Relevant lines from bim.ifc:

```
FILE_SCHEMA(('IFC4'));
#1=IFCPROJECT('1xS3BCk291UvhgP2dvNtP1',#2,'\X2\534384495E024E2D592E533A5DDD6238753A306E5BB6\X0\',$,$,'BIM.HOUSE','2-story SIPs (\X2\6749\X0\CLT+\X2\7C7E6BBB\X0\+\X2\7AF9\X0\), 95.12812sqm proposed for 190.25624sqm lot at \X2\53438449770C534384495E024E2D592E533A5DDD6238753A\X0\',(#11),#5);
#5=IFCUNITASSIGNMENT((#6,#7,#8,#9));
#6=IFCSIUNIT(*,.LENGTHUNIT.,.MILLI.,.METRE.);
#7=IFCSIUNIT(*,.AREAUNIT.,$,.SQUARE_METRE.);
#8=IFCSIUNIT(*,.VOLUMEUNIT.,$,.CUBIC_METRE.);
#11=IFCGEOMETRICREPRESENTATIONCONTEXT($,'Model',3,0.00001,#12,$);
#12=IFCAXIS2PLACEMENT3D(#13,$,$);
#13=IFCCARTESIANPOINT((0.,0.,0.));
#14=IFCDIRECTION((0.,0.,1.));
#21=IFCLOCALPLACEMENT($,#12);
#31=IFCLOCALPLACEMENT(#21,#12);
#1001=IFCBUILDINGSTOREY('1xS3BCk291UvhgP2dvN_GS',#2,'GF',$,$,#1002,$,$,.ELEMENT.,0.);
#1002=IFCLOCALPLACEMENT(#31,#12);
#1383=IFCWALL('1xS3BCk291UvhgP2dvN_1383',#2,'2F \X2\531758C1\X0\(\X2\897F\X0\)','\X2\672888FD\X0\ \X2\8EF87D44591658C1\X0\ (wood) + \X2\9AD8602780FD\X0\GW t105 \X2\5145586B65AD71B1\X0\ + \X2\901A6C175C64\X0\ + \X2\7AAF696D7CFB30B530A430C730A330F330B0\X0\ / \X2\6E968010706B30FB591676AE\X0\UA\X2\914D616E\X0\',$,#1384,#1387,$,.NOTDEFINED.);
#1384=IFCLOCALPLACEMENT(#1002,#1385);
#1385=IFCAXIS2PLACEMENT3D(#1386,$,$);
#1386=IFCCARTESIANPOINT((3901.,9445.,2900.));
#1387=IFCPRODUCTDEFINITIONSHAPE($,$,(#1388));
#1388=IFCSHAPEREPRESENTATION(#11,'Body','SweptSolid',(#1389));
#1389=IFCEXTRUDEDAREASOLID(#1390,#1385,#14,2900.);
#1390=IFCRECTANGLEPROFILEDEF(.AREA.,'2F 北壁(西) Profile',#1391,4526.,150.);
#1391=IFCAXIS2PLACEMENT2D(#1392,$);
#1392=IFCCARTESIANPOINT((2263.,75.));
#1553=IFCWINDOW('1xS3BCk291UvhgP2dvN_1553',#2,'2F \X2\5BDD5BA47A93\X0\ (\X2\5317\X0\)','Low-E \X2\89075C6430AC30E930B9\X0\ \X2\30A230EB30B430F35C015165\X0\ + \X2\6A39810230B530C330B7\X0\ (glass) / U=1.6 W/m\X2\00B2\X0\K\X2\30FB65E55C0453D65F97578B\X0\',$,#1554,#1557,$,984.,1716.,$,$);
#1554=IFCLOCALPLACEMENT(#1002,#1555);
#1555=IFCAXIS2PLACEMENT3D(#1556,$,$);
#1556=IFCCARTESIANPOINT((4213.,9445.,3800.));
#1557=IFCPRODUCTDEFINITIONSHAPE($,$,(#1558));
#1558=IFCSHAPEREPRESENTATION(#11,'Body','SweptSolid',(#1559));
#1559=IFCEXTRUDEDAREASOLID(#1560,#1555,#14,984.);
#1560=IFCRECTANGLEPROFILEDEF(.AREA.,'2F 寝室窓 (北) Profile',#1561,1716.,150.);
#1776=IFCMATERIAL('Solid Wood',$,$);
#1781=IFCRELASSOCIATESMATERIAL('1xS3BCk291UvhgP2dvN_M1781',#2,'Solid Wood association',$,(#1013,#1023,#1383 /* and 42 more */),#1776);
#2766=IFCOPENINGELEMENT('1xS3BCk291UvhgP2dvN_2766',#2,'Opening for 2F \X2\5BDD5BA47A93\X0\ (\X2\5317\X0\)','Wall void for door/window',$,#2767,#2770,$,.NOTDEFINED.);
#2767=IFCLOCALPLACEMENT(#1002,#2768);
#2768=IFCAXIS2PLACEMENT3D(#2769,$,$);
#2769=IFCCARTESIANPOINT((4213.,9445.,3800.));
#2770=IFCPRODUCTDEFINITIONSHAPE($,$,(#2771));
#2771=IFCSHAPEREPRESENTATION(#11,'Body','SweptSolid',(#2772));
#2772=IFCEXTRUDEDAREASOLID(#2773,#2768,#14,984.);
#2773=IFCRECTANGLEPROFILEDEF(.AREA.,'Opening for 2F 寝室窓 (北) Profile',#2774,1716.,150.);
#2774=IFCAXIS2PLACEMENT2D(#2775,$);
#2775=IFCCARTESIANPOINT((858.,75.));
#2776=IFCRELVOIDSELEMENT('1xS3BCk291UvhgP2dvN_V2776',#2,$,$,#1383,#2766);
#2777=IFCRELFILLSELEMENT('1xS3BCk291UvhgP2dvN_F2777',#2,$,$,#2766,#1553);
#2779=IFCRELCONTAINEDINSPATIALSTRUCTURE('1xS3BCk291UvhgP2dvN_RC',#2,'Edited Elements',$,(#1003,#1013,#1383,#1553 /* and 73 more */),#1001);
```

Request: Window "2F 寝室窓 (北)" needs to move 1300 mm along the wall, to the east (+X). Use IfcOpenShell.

```python
import ifcopenshell
import ifcopenshell.api.geometry
import ifcopenshell.util.placement
import ifcopenshell.util.unit

model = ifcopenshell.open("bim.ifc")
unit_scale = ifcopenshell.util.unit.calculate_unit_scale(model)

window = model.by_guid("1xS3BCk291UvhgP2dvN_1553")
opening = window.FillsVoids[0].RelatingOpeningElement
wall = opening.VoidsElements[0].RelatingBuildingElement

wall_matrix = ifcopenshell.util.placement.get_local_placement(wall.ObjectPlacement)
shift = wall_matrix[:3, 0] * 1.3 / unit_scale
before = ifcopenshell.util.placement.get_local_placement(window.ObjectPlacement)[:3, 3].copy()

# The window is not placed relative to its opening, so move both.
for product in (opening, window):
    matrix = ifcopenshell.util.placement.get_local_placement(product.ObjectPlacement)
    matrix[:3, 3] += shift
    ifcopenshell.api.geometry.edit_object_placement(model, product=product, matrix=matrix, is_si=False)

after = ifcopenshell.util.placement.get_local_placement(window.ObjectPlacement)[:3, 3]
print("window moved by", (after - before).round(3) + 0.0)

model.write("bim_rev.ifc")
```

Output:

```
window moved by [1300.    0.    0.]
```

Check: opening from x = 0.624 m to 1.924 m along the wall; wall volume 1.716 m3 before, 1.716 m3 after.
